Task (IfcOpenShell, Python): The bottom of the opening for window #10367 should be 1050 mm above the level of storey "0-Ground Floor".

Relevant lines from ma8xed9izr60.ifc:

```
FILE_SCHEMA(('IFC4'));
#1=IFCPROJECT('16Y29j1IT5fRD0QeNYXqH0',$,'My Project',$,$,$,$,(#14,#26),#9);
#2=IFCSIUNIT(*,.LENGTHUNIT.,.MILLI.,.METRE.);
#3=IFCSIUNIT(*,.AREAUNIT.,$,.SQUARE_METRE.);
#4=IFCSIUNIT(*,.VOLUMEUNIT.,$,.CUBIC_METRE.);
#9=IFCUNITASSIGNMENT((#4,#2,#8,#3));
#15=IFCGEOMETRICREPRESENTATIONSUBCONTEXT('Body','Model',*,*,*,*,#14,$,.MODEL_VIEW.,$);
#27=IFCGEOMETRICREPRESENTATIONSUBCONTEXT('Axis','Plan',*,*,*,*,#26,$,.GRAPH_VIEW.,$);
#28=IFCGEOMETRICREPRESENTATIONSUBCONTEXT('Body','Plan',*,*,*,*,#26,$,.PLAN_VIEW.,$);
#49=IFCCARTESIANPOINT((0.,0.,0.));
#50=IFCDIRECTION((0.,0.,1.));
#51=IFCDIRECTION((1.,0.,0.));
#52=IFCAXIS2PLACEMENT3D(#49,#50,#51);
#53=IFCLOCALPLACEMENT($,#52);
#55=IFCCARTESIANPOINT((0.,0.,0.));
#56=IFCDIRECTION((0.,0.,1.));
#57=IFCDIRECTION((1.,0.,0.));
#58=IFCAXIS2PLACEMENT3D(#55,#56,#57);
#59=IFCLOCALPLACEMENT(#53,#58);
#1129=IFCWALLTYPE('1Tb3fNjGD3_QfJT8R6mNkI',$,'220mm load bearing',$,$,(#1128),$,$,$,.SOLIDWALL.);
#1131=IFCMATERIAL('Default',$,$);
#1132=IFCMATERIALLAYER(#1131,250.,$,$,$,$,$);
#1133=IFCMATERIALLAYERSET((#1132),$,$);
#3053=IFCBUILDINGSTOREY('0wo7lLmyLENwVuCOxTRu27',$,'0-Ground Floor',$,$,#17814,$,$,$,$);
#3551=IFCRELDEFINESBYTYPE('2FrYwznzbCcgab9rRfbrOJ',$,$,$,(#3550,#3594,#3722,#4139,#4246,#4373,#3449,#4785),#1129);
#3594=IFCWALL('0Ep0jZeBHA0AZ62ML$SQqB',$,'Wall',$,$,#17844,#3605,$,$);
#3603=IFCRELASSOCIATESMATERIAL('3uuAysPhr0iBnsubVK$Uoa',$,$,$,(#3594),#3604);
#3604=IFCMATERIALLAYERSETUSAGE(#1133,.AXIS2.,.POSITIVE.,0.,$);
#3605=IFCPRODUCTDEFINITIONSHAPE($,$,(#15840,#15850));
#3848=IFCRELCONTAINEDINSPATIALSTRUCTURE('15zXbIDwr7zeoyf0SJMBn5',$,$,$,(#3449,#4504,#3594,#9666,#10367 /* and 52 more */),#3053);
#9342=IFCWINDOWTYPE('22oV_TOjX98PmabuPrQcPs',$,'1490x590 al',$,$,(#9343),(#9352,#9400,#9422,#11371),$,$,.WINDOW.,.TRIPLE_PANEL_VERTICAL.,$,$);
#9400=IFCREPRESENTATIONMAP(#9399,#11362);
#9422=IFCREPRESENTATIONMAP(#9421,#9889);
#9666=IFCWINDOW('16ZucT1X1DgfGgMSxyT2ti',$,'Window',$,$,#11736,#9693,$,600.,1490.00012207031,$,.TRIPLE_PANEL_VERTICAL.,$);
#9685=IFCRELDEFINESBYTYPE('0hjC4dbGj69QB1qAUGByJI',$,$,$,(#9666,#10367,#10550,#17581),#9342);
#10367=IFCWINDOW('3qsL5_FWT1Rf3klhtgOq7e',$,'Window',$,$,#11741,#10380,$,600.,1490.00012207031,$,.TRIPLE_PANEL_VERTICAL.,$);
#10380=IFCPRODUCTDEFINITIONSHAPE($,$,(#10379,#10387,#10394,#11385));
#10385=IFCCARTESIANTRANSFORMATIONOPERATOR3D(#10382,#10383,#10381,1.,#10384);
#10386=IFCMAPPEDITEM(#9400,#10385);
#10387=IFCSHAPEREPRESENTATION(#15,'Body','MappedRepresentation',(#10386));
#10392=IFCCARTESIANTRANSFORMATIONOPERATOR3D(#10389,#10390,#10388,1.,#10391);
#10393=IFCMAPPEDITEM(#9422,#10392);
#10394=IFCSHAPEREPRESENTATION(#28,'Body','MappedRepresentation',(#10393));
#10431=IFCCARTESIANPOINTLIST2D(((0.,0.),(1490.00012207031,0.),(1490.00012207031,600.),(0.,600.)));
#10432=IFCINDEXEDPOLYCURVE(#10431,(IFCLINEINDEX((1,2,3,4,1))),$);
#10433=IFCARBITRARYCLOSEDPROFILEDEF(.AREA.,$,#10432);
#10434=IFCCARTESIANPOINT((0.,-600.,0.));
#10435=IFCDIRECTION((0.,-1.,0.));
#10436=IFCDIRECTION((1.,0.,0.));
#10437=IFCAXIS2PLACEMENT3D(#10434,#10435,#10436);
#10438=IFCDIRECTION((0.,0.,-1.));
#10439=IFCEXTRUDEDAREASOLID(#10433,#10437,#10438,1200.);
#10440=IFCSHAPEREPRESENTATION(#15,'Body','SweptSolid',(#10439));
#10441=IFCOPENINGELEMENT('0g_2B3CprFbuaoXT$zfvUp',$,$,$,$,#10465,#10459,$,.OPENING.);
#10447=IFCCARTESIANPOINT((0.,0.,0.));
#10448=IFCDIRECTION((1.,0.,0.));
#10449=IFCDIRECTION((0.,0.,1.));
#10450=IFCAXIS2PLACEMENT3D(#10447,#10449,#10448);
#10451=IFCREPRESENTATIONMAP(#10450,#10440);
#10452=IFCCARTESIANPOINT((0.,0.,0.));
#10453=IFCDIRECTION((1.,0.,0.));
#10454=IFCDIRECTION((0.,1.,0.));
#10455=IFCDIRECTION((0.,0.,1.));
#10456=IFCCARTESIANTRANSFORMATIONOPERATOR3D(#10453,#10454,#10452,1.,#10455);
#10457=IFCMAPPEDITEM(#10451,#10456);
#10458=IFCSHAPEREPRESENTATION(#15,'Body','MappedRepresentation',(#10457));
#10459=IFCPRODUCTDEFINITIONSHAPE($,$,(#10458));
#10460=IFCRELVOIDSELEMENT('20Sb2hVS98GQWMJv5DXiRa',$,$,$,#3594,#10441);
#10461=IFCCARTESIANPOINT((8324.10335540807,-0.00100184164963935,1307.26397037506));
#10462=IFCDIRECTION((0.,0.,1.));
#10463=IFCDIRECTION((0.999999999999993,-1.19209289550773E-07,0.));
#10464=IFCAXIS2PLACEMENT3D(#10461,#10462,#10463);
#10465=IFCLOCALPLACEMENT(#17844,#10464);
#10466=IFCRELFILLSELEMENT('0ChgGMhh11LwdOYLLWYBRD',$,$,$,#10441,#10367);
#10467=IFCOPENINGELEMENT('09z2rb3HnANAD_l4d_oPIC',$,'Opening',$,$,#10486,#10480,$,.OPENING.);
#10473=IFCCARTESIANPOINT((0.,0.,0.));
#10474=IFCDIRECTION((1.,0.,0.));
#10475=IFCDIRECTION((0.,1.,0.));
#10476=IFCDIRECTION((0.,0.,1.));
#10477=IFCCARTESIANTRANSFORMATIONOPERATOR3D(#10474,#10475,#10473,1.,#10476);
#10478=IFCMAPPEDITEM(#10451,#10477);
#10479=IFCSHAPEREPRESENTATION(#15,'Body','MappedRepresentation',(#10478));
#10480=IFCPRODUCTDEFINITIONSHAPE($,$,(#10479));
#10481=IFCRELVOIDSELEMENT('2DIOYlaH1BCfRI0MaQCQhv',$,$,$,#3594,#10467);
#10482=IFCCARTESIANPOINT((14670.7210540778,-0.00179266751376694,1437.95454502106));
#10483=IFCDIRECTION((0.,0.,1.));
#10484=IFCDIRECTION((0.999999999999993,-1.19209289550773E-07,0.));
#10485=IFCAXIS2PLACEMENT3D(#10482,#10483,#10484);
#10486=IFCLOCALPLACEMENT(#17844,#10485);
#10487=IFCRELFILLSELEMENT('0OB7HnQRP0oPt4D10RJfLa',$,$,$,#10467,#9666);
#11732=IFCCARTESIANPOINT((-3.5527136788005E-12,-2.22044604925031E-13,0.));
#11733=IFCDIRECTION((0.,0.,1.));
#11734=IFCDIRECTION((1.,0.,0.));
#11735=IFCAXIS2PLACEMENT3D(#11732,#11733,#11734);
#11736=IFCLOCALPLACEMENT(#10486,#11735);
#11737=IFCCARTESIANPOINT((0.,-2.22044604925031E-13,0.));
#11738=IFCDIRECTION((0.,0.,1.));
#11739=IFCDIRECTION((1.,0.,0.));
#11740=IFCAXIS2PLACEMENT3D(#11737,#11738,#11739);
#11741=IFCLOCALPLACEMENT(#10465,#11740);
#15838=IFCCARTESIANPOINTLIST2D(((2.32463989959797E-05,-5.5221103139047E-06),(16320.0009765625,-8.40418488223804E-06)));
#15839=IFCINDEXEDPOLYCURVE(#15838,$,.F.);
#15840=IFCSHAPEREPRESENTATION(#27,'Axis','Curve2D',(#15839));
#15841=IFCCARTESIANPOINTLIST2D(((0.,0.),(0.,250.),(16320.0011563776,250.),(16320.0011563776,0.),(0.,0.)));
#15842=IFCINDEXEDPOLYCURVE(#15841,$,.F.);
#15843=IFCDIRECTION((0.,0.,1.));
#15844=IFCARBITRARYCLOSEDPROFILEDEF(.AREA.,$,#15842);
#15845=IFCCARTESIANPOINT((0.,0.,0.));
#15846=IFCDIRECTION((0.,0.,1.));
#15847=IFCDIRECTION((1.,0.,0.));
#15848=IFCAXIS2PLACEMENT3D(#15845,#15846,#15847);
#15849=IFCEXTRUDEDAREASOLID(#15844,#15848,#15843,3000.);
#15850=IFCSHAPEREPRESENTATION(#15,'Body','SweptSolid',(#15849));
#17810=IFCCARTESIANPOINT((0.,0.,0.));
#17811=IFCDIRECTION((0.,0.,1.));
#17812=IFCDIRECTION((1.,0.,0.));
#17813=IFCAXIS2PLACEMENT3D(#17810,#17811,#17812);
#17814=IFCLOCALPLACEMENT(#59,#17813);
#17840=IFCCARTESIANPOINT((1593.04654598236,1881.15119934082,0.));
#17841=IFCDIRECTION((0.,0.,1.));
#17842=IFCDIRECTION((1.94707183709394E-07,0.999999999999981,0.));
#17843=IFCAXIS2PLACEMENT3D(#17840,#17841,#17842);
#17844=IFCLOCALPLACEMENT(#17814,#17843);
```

```python
import numpy as np
import ifcopenshell
import ifcopenshell.api.geometry
import ifcopenshell.geom
import ifcopenshell.util.element
import ifcopenshell.util.placement
import ifcopenshell.util.shape
import ifcopenshell.util.unit

model = ifcopenshell.open("ma8xed9izr60.ifc")
unit_scale = ifcopenshell.util.unit.calculate_unit_scale(model)

window = model.by_id(10367)
opening = window.FillsVoids[0].RelatingOpeningElement
storey = ifcopenshell.util.element.get_container(window, ifc_class="IfcBuildingStorey")
level = ifcopenshell.util.placement.get_local_placement(storey.ObjectPlacement)[2, 3]

# The opening's origin need not be at the sill, so measure its lowest point.
shape = ifcopenshell.geom.create_shape(ifcopenshell.geom.settings(), opening)
bottom = ifcopenshell.util.shape.get_shape_bottom_elevation(shape, shape.geometry) / unit_scale
dz = level + 1.05 / unit_scale - bottom

shift = np.array([0.0, 0.0, dz])
# The window is placed relative to its opening, so it follows when the opening moves.
matrix = ifcopenshell.util.placement.get_local_placement(opening.ObjectPlacement)
matrix[:3, 3] += shift
ifcopenshell.api.geometry.edit_object_placement(
    model, product=opening, matrix=matrix, is_si=False, should_transform_children=True
)

print(f"moved by {dz * unit_scale:+.3f} m")

model.write("ma8xed9izr60_updated.ifc")
```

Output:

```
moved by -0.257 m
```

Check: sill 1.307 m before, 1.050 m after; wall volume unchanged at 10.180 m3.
